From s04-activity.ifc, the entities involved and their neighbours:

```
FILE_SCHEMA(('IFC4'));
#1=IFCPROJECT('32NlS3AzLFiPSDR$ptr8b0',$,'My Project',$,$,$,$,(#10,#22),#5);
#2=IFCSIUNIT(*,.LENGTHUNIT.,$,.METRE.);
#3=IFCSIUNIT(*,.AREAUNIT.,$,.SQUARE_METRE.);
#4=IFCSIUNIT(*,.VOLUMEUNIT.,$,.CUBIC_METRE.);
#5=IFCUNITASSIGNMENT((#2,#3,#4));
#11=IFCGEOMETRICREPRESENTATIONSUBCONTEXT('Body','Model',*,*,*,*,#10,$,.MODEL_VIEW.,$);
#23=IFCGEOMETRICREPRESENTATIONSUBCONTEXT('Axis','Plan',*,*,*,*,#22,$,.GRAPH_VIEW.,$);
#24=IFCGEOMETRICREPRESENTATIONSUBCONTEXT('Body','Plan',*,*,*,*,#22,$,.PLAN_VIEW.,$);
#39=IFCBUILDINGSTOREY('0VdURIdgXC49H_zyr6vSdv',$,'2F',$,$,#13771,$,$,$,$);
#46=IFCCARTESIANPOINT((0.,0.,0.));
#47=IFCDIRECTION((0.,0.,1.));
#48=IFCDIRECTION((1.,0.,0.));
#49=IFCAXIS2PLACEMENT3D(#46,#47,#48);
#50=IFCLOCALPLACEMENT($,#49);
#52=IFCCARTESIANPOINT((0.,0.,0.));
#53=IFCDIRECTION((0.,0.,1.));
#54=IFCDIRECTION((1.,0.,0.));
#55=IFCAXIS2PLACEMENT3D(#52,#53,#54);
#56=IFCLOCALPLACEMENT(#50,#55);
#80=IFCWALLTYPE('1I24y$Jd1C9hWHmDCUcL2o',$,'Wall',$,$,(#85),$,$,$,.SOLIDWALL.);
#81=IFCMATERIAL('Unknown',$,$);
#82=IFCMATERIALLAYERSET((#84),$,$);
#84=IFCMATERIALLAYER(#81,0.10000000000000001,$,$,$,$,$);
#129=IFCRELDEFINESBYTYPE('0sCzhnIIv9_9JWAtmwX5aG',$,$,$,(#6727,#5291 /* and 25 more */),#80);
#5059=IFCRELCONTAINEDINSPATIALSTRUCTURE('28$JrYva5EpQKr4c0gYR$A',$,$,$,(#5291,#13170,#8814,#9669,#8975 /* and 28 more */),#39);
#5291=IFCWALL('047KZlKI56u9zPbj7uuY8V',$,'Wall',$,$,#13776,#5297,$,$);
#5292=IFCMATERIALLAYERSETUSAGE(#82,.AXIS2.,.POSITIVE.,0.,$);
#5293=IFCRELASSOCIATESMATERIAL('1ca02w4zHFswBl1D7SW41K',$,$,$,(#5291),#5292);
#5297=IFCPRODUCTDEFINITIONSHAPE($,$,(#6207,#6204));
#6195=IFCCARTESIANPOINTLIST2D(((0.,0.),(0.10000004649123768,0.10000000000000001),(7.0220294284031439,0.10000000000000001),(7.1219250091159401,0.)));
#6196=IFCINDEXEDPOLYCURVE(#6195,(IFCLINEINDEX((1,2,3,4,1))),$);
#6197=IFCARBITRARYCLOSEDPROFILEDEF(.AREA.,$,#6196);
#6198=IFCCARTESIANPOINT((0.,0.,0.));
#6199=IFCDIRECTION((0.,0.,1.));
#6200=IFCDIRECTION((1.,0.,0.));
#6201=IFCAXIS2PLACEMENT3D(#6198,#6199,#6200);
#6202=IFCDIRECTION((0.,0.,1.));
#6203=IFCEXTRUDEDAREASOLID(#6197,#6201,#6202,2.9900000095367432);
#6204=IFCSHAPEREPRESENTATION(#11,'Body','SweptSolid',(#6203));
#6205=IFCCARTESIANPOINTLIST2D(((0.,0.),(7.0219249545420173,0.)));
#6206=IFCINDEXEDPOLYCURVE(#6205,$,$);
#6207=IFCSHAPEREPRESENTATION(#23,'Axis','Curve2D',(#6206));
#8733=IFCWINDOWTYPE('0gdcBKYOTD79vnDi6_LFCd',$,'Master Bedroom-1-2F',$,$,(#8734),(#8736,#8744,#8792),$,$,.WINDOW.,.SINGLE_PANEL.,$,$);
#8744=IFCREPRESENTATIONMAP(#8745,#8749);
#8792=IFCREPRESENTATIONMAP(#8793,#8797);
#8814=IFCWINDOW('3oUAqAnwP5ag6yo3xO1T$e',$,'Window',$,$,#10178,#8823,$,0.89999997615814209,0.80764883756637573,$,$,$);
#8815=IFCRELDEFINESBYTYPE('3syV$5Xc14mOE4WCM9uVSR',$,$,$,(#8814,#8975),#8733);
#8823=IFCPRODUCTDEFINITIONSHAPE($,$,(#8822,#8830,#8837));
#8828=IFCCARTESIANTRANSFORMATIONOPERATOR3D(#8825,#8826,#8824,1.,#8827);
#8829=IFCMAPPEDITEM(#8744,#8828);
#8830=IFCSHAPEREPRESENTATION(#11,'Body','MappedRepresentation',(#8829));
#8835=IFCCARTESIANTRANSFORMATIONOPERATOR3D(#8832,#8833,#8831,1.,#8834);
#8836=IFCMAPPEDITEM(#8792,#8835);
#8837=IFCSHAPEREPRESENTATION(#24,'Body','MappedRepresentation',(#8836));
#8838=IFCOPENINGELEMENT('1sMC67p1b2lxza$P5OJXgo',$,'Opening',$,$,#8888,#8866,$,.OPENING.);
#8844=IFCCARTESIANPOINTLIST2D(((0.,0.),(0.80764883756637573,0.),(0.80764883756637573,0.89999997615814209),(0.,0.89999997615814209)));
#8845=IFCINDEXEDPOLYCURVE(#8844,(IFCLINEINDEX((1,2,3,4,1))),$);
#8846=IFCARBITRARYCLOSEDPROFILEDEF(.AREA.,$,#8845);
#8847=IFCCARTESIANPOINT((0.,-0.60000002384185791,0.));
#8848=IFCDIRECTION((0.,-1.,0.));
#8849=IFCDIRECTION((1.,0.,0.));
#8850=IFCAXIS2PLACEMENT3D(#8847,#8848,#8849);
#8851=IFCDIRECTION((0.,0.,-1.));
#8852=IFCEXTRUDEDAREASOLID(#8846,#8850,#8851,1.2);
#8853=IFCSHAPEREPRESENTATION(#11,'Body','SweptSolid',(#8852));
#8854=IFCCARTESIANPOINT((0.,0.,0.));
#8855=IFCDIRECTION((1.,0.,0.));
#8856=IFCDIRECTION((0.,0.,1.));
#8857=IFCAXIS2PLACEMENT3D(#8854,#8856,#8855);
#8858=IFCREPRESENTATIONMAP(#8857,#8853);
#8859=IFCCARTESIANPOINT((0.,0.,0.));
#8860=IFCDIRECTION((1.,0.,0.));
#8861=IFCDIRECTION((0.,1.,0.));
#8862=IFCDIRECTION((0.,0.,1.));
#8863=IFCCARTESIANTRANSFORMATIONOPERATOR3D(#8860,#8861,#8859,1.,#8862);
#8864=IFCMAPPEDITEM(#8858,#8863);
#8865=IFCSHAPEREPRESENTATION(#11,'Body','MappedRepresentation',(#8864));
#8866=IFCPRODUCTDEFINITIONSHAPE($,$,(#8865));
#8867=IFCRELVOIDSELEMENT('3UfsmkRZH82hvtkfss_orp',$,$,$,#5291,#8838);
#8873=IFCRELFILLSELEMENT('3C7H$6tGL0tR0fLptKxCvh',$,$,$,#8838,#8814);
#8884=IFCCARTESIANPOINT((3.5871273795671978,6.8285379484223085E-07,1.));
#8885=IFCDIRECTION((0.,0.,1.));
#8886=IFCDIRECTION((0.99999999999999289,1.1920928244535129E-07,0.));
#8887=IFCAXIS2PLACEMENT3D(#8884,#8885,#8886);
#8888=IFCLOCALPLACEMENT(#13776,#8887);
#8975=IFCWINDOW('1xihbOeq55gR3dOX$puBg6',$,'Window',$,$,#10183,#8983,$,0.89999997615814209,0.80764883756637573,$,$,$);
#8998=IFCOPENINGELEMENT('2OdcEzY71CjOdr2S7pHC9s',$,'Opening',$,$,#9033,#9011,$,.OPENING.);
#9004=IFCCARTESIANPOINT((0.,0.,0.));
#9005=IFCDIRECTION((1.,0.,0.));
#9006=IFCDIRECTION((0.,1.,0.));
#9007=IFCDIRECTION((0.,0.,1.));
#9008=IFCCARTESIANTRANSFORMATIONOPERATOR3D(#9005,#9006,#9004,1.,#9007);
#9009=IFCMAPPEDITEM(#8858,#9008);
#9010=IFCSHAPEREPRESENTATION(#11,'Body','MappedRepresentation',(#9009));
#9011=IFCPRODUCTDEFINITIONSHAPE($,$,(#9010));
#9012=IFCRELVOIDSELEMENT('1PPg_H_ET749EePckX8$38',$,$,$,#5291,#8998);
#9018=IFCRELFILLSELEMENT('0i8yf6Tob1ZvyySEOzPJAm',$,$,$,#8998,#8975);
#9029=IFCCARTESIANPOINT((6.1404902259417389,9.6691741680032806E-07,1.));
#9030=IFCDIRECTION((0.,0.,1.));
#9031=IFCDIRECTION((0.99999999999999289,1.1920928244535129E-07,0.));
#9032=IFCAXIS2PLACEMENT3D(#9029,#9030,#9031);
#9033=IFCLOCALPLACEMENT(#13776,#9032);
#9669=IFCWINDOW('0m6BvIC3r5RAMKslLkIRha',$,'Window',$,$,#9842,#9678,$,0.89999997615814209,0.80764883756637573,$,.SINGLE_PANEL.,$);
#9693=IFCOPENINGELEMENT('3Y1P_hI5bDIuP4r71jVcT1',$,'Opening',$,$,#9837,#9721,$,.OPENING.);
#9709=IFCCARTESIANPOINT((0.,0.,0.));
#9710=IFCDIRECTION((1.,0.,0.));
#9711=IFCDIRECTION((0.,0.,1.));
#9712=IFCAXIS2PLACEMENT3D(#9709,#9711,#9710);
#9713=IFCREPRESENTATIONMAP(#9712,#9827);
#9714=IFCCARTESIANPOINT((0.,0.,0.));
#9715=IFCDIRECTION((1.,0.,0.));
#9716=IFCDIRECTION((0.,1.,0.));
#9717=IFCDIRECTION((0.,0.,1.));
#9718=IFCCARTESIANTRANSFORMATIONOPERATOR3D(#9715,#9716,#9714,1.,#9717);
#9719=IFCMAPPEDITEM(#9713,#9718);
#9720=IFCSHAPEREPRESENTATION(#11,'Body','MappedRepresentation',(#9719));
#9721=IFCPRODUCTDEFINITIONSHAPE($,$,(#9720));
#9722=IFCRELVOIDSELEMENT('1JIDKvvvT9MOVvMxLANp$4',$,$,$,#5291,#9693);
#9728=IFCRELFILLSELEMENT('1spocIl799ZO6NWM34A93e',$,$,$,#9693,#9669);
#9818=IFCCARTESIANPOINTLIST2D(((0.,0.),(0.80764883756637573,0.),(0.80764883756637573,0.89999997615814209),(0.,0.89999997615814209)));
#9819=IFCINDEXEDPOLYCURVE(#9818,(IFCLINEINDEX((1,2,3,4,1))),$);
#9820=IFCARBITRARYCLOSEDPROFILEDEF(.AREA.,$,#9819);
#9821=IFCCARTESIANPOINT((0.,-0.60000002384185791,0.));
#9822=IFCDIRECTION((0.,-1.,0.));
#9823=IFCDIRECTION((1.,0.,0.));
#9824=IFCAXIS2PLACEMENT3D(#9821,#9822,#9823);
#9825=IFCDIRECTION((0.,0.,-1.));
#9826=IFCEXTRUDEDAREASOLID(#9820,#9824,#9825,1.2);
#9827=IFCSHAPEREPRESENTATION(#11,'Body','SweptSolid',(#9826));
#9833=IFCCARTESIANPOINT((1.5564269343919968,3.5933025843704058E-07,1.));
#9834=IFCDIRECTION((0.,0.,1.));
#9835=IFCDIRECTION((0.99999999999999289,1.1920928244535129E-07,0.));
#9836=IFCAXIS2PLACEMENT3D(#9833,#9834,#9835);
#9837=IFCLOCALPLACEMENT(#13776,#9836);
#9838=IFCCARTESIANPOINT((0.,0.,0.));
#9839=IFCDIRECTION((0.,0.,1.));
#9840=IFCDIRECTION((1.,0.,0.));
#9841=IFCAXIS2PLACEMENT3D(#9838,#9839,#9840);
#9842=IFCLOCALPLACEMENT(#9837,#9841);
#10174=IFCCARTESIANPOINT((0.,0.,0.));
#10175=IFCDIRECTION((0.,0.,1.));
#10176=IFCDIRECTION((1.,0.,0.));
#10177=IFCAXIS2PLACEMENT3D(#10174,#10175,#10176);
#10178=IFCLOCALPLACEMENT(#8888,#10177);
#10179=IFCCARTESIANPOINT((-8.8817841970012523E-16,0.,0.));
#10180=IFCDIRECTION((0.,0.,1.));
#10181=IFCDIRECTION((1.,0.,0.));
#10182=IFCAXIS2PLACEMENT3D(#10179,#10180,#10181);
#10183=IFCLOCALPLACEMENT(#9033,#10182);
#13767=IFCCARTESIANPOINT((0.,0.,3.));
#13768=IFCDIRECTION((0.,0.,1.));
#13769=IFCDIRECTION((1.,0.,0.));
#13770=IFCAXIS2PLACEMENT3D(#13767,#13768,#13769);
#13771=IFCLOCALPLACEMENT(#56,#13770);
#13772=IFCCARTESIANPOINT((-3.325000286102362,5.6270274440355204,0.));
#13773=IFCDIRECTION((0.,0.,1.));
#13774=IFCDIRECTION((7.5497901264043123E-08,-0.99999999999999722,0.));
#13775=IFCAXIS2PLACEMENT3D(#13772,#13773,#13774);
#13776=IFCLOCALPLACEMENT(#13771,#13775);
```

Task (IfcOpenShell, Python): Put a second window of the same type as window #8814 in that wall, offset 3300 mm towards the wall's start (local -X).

```python
import ifcopenshell
import ifcopenshell.api.feature
import ifcopenshell.api.geometry
import ifcopenshell.api.root
import ifcopenshell.geom
import ifcopenshell.util.element
import ifcopenshell.util.placement
import ifcopenshell.util.shape
import ifcopenshell.util.unit

model = ifcopenshell.open("s04-activity.ifc")
unit_scale = ifcopenshell.util.unit.calculate_unit_scale(model)
settings = ifcopenshell.geom.settings()


def volume(element):
    """Net volume in cubic metres, openings subtracted."""
    shape = ifcopenshell.geom.create_shape(settings, element)
    return ifcopenshell.util.shape.get_volume(shape.geometry)


window = model.by_id(8814)
opening = window.FillsVoids[0].RelatingOpeningElement
wall = opening.VoidsElements[0].RelatingBuildingElement
before = volume(wall)
shift = ifcopenshell.util.placement.get_local_placement(wall.ObjectPlacement)[:3, 0] * -3.3 / unit_scale

# copy_class copies the void relationship, type, container and properties, but no geometry.
new_opening = ifcopenshell.api.root.copy_class(model, product=opening)
new_opening.Representation = ifcopenshell.util.element.copy_deep(
    model, opening.Representation, exclude=["IfcGeometricRepresentationContext", "IfcRepresentationMap"]
)
new_window = ifcopenshell.api.root.copy_class(model, product=window)
new_window.Representation = ifcopenshell.util.element.copy_deep(
    model, window.Representation, exclude=["IfcGeometricRepresentationContext", "IfcRepresentationMap"]
)
ifcopenshell.api.feature.add_filling(model, opening=new_opening, element=new_window)

for old, new in ((opening, new_opening), (window, new_window)):
    matrix = ifcopenshell.util.placement.get_local_placement(old.ObjectPlacement)
    matrix[:3, 3] += shift
    ifcopenshell.api.geometry.edit_object_placement(model, product=new, matrix=matrix, is_si=False)

after = volume(wall)

print(f"wall volume {before:.3f} -> {after:.3f} m3")

model.write("s04-activity-out.ifc")
```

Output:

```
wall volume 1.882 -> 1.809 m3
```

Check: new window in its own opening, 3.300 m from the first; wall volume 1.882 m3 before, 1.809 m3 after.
